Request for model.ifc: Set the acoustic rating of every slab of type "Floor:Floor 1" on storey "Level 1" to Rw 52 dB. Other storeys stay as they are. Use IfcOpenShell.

First a look at what the model holds.

```python
import ifcopenshell
import ifcopenshell.util.element

model = ifcopenshell.open("model.ifc")
print(model.schema)
storey = next(s for s in model.by_type("IfcBuildingStorey") if s.Name == "Level 1")
slabs = [e for e in ifcopenshell.util.element.get_decomposition(storey) if e.is_a("IfcSlab")]
seen = {}
for e in slabs:
    element_type = ifcopenshell.util.element.get_type(e)
    key = (element_type.Name if element_type != e and element_type else None, ifcopenshell.util.element.get_pset(e, "Pset_SlabCommon", "AcousticRating"))
    seen[key] = seen.get(key, 0) + 1
for (name, value), count in sorted(seen.items(), key=str):
    print(count, "x", name, "|", value)
```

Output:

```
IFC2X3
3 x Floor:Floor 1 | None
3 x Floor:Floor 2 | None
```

```python
import ifcopenshell
import ifcopenshell.api.pset
import ifcopenshell.util.element

model = ifcopenshell.open("model.ifc")

storey = next(s for s in model.by_type("IfcBuildingStorey") if s.Name == "Level 1")
slabs = [e for e in ifcopenshell.util.element.get_decomposition(storey) if e.is_a("IfcSlab")]

count = 0
for e in slabs:
    element_type = ifcopenshell.util.element.get_type(e)
    if element_type in (None, e) or element_type.Name != "Floor:Floor 1":
        continue
    # add_pset returns the element's existing set when there is one.
    pset = ifcopenshell.api.pset.add_pset(model, product=e, name="Pset_SlabCommon")
    ifcopenshell.api.pset.edit_pset(model, pset=pset, properties={"AcousticRating": "Rw 52 dB"})
    count += 1

print(count, "slabs updated")

model.write("model_v2.ifc")
```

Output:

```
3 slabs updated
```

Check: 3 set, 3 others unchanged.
